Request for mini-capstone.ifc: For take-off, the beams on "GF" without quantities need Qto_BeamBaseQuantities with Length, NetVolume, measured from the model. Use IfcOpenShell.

First a look at what the model holds.

```python
import ifcopenshell
import ifcopenshell.util.element
import ifcopenshell.util.unit

model = ifcopenshell.open("mini-capstone.ifc")
print(model.schema)
for unit_type in ("LENGTHUNIT", "AREAUNIT", "VOLUMEUNIT"):
    print(unit_type, ifcopenshell.util.unit.calculate_unit_scale(model, unit_type))
storey = next(s for s in model.by_type("IfcBuildingStorey") if s.Name == "GF")
beams = [e for e in ifcopenshell.util.element.get_decomposition(storey) if e.is_a("IfcBeam")]
for e in sorted(beams, key=lambda e: e.id()):
    print(e.id(), e.is_a(), e.Name, list(ifcopenshell.util.element.get_psets(e, qtos_only=True)), sep=" | ")
```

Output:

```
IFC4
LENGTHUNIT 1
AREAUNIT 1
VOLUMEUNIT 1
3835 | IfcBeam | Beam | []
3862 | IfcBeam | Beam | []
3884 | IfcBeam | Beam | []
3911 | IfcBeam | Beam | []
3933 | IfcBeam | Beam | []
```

```python
import ifcopenshell
import ifcopenshell.api.pset
import ifcopenshell.geom
import ifcopenshell.util.element
import ifcopenshell.util.shape
import ifcopenshell.util.unit

model = ifcopenshell.open("mini-capstone.ifc")
unit_scale = ifcopenshell.util.unit.calculate_unit_scale(model)
volume_scale = ifcopenshell.util.unit.calculate_unit_scale(model, "VOLUMEUNIT")
settings = ifcopenshell.geom.settings()

storey = next(s for s in model.by_type("IfcBuildingStorey") if s.Name == "GF")
beams = [e for e in ifcopenshell.util.element.get_decomposition(storey) if e.is_a("IfcBeam")]

for e in sorted(beams, key=lambda e: e.id()):
    if ifcopenshell.util.element.get_psets(e, qtos_only=True, should_inherit=False):
        continue
    # Geometry comes back in metres, in the element's own axes.
    shape = ifcopenshell.geom.create_shape(settings, e)
    values = {
        "Length": ifcopenshell.util.shape.get_max_xyz(shape.geometry) / unit_scale,
        "NetVolume": ifcopenshell.util.shape.get_volume(shape.geometry) / volume_scale,
    }
    qto = ifcopenshell.api.pset.add_qto(model, product=e, name="Qto_BeamBaseQuantities")
    ifcopenshell.api.pset.edit_qto(model, qto=qto, properties=values)
    print(e.id(), {k: round(v, 3) for k, v in values.items()})

model.write("mini-capstone_rev.ifc")
```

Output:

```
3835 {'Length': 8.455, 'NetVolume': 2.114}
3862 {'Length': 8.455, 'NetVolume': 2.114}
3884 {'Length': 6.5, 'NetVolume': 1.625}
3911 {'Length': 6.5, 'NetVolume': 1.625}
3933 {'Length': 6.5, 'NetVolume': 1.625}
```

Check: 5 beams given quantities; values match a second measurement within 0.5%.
